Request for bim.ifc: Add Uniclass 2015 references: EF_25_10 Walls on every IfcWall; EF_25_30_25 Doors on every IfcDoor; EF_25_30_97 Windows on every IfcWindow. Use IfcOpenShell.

First a look at what the model holds.

```python
import ifcopenshell

model = ifcopenshell.open("bim.ifc")
print(model.schema)
print("classifications:", [c.Name for c in model.by_type("IfcClassification")])
for ifc_class in ("IfcDoor", "IfcRoof", "IfcStair", "IfcWall", "IfcWindow"):
    print(ifc_class, len(model.by_type(ifc_class)))
```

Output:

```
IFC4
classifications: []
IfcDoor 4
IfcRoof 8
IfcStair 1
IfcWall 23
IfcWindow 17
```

```python
import ifcopenshell
import ifcopenshell.api.classification

model = ifcopenshell.open("bim.ifc")

system = ifcopenshell.api.classification.add_classification(model, classification="Uniclass 2015")

codes = {
    "IfcWall": ("EF_25_10", "Walls"),
    "IfcDoor": ("EF_25_30_25", "Doors"),
    "IfcWindow": ("EF_25_30_97", "Windows"),
}
for ifc_class, (code, name) in codes.items():
    products = model.by_type(ifc_class)
    ifcopenshell.api.classification.add_reference(
        model, products=products, classification=system, identification=code, name=name
    )
    print(code, len(products))

model.write("bim-out.ifc")
```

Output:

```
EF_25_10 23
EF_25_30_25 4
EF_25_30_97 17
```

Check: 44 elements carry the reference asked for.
